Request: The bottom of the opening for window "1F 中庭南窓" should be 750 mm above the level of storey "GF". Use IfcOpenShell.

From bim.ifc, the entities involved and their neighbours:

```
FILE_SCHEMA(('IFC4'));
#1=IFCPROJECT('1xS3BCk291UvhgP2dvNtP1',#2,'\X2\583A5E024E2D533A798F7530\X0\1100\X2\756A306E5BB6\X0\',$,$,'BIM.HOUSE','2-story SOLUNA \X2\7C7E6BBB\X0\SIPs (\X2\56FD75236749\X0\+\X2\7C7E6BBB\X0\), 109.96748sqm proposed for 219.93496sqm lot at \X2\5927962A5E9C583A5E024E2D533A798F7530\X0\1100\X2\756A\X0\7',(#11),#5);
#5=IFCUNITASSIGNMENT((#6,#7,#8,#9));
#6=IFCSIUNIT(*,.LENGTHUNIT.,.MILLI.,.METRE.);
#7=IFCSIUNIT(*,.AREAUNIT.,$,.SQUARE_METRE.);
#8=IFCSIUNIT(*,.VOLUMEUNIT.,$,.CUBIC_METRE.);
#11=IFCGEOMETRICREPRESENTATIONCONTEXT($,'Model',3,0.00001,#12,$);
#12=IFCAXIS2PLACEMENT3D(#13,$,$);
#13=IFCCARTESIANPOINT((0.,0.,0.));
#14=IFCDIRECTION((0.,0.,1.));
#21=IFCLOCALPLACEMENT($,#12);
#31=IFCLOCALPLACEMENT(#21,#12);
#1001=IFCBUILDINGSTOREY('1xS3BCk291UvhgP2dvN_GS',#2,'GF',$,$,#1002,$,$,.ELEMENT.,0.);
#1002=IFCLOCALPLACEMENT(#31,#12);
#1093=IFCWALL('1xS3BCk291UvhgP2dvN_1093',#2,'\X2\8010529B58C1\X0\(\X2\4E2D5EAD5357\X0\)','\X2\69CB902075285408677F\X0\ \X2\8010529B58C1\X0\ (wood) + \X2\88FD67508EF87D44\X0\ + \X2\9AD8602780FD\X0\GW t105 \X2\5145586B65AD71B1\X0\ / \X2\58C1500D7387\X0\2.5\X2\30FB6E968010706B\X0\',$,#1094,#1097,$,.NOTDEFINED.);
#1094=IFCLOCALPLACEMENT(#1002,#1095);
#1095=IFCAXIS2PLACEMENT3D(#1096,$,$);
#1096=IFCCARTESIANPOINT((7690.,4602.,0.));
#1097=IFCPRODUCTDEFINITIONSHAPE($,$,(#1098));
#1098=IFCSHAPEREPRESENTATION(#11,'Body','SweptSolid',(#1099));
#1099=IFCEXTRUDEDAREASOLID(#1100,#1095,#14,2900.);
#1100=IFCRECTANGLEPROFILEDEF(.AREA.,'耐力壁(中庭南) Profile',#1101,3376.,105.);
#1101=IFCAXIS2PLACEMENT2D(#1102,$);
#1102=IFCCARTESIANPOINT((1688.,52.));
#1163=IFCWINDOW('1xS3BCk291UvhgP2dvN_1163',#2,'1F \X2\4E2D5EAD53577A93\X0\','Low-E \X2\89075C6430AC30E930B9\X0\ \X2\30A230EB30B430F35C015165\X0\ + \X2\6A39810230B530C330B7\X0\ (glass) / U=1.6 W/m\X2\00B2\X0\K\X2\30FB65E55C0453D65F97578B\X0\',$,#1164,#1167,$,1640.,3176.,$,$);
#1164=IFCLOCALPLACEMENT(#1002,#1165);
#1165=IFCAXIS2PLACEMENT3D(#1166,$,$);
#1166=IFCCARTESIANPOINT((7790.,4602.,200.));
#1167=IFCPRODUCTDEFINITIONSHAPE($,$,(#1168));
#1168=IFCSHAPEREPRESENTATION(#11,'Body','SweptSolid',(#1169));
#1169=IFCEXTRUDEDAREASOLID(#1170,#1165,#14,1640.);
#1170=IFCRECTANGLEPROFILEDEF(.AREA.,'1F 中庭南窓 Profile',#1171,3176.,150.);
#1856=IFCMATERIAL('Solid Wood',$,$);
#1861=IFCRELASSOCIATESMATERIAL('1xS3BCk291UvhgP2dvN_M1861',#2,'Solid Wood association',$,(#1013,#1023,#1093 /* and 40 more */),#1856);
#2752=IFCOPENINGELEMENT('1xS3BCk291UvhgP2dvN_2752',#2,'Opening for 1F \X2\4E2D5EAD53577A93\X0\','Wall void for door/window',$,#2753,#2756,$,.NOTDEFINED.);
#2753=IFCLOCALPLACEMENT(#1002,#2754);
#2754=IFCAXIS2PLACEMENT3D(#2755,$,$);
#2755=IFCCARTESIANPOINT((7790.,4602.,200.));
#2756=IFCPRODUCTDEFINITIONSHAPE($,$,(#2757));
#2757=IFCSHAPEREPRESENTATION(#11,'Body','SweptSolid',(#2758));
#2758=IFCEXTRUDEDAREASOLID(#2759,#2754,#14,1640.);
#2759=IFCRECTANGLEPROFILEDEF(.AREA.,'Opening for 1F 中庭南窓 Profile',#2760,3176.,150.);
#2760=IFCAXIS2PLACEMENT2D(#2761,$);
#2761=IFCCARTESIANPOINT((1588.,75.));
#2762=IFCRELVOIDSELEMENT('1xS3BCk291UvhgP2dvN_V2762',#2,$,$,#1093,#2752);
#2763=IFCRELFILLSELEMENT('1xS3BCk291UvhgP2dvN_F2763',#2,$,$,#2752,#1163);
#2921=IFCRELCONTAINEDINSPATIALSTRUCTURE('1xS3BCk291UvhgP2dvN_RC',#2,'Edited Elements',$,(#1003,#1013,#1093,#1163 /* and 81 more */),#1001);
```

```python
import numpy as np
import ifcopenshell
import ifcopenshell.api.geometry
import ifcopenshell.geom
import ifcopenshell.util.element
import ifcopenshell.util.placement
import ifcopenshell.util.shape
import ifcopenshell.util.unit

model = ifcopenshell.open("bim.ifc")
unit_scale = ifcopenshell.util.unit.calculate_unit_scale(model)

window = model.by_guid("1xS3BCk291UvhgP2dvN_1163")
opening = window.FillsVoids[0].RelatingOpeningElement
storey = ifcopenshell.util.element.get_container(window, ifc_class="IfcBuildingStorey")
level = ifcopenshell.util.placement.get_local_placement(storey.ObjectPlacement)[2, 3]

# The opening's origin need not be at the sill, so measure its lowest point.
shape = ifcopenshell.geom.create_shape(ifcopenshell.geom.settings(), opening)
bottom = ifcopenshell.util.shape.get_shape_bottom_elevation(shape, shape.geometry) / unit_scale
dz = level + 0.75 / unit_scale - bottom

shift = np.array([0.0, 0.0, dz])
# The window is not placed relative to its opening, so move both.
for product in (opening, window):
    matrix = ifcopenshell.util.placement.get_local_placement(product.ObjectPlacement)
    matrix[:3, 3] += shift
    ifcopenshell.api.geometry.edit_object_placement(model, product=product, matrix=matrix, is_si=False)

print(f"moved by {dz * unit_scale:+.3f} m")

model.write("bim_v2.ifc")
```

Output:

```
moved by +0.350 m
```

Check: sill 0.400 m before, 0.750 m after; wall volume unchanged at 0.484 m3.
